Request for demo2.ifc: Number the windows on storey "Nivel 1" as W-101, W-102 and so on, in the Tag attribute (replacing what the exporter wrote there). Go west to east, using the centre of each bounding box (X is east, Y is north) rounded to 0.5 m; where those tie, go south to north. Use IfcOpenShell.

First a look at what the model holds.

```python
import ifcopenshell
import ifcopenshell.util.element
import ifcopenshell.util.placement

model = ifcopenshell.open("demo2.ifc")
print(model.schema)
storey = next(s for s in model.by_type("IfcBuildingStorey") if s.Name == "Nivel 1")
windows = [e for e in ifcopenshell.util.element.get_decomposition(storey) if e.is_a("IfcWindow")]
for e in sorted(windows, key=lambda e: e.id()):
    origin = ifcopenshell.util.placement.get_local_placement(e.ObjectPlacement)[:3, 3]
    print(e.id(), e.Tag, e.Name, origin.round(2) + 0.0, sep=" | ")
```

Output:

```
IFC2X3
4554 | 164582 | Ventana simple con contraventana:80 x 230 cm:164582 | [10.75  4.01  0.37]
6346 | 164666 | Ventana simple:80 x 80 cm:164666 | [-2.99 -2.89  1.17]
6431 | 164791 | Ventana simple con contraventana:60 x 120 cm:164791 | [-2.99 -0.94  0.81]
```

```python
import ifcopenshell
import ifcopenshell.geom
import ifcopenshell.util.element
import ifcopenshell.util.shape

model = ifcopenshell.open("demo2.ifc")
settings = ifcopenshell.geom.settings()
settings.set("use-world-coords", True)


def centre(element):
    shape = ifcopenshell.geom.create_shape(settings, element)
    return ifcopenshell.util.shape.get_bbox_centroid(shape.geometry)


storey = next(s for s in model.by_type("IfcBuildingStorey") if s.Name == "Nivel 1")
windows = [e for e in ifcopenshell.util.element.get_decomposition(storey) if e.is_a("IfcWindow")]

# Insertion points can sit at a corner or the storey origin, so sort by the geometry (in metres).
centres = {e: centre(e) for e in windows}
windows.sort(key=lambda e: (round(centres[e][0] / 0.5), centres[e][1]))

for i, e in enumerate(windows, start=1):
    number = f"W-1{i:02d}"
    e.Tag = number
    print(e.id(), number)

model.write("demo2_updated.ifc")
```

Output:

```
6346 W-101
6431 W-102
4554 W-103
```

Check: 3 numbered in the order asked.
